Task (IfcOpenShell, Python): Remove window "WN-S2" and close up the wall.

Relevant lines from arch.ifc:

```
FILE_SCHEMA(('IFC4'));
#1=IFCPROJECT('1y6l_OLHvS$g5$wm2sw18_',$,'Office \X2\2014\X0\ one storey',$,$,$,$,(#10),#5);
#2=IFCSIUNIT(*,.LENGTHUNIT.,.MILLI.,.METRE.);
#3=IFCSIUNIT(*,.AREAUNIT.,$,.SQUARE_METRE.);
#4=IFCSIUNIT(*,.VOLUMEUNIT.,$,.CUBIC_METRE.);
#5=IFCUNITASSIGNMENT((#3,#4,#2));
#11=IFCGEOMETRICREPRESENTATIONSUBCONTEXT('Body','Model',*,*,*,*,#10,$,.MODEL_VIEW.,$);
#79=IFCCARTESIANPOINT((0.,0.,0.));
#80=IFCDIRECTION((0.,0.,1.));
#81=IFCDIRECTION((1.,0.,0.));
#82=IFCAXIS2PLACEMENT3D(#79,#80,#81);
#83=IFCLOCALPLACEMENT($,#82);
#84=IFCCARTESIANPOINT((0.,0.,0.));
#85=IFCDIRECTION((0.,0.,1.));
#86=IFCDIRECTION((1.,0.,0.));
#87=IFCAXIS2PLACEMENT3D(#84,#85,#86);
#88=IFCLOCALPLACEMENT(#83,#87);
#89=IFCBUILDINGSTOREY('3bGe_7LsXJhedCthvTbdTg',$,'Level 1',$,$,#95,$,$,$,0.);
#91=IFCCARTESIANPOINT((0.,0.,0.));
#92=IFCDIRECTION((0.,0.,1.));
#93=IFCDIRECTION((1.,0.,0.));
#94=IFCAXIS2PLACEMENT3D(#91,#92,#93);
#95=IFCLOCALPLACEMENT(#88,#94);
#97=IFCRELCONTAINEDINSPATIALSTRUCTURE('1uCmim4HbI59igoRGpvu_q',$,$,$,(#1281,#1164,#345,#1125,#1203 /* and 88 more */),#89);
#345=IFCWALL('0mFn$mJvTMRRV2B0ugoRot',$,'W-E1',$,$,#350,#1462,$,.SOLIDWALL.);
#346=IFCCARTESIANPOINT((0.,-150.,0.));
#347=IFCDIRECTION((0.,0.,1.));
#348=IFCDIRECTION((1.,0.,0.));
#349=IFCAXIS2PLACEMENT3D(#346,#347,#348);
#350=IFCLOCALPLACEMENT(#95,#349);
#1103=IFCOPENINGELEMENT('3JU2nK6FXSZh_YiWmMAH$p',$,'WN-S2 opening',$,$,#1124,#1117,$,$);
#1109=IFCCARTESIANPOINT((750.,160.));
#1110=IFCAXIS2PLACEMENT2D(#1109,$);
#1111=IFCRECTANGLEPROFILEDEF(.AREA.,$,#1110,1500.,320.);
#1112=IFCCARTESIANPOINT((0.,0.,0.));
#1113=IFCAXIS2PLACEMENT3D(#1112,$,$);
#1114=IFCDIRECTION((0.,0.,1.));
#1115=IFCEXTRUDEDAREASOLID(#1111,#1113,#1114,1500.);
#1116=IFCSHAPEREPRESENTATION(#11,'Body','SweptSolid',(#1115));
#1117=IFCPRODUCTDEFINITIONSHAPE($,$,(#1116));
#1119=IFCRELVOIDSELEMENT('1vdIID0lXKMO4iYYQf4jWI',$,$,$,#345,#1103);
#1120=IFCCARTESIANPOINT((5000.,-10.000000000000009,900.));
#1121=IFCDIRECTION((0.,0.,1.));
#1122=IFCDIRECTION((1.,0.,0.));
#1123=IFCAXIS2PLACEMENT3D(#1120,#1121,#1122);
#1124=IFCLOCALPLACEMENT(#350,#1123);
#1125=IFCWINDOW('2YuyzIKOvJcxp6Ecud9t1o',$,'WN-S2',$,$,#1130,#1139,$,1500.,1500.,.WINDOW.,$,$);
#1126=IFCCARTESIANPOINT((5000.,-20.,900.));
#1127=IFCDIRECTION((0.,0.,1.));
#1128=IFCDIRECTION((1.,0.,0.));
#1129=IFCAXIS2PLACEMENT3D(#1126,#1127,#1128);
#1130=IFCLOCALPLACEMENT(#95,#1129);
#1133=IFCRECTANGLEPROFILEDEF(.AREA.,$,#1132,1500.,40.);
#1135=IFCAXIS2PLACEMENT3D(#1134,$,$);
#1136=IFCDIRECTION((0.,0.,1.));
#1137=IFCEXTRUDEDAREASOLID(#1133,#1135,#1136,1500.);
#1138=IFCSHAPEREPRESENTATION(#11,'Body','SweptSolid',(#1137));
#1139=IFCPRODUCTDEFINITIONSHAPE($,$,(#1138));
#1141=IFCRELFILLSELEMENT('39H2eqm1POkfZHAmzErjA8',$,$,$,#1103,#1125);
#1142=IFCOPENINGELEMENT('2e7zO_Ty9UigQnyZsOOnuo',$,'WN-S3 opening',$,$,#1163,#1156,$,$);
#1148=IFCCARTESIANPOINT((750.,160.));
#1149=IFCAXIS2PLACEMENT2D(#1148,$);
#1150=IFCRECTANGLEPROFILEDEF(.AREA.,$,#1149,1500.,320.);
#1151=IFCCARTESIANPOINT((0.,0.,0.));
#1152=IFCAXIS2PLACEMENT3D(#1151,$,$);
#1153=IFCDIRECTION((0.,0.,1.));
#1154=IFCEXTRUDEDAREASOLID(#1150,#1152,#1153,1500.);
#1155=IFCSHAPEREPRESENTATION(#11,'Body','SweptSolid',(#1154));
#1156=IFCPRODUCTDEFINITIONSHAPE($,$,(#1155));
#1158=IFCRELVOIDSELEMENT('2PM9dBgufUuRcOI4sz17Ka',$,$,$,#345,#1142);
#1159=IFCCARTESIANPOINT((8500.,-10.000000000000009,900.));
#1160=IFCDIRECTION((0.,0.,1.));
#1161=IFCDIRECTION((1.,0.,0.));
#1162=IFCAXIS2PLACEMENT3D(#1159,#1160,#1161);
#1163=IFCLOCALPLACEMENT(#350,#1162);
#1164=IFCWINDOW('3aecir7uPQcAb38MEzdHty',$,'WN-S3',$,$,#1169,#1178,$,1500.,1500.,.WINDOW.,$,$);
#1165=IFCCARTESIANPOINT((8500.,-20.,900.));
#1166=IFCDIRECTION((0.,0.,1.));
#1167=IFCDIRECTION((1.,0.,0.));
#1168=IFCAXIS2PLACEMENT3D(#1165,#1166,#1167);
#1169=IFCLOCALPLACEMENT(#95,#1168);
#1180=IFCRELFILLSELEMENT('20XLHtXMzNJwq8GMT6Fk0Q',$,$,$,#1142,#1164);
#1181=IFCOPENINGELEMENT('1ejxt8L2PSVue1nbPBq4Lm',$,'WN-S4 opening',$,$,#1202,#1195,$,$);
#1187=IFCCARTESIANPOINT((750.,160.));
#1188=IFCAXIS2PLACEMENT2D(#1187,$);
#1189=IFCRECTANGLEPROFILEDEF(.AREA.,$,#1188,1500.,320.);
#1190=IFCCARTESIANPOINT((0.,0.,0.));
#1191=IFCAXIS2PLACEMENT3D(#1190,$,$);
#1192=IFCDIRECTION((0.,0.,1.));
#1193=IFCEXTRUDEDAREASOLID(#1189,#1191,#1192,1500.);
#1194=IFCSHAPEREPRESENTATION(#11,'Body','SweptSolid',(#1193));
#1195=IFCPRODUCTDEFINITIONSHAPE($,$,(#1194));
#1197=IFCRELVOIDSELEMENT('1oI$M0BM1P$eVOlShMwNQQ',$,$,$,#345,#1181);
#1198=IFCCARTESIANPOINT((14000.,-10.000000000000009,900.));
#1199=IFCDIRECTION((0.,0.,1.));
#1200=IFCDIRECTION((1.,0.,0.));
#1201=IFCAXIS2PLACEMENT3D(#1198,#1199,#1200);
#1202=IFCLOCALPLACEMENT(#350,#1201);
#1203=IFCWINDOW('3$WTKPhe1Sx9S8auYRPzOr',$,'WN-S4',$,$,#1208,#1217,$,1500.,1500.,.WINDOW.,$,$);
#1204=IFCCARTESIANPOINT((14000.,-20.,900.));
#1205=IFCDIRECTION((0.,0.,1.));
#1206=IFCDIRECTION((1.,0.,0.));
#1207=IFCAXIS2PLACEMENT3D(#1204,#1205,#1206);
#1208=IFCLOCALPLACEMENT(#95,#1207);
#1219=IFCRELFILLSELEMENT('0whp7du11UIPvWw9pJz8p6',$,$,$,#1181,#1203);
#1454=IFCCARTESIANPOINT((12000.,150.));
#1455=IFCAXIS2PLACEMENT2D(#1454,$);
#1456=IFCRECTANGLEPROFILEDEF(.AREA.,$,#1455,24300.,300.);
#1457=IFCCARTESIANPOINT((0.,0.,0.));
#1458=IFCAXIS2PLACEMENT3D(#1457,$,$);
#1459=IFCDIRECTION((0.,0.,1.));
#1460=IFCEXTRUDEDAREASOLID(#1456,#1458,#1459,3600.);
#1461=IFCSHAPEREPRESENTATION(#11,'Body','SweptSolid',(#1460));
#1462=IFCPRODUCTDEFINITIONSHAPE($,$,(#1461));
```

```python
import ifcopenshell
import ifcopenshell.api.feature
import ifcopenshell.api.root
import ifcopenshell.geom
import ifcopenshell.util.shape

model = ifcopenshell.open("arch.ifc")
settings = ifcopenshell.geom.settings()


def volume(element):
    """Net volume in cubic metres, openings subtracted."""
    shape = ifcopenshell.geom.create_shape(settings, element)
    return ifcopenshell.util.shape.get_volume(shape.geometry)


window = model.by_guid("2YuyzIKOvJcxp6Ecud9t1o")
opening = window.FillsVoids[0].RelatingOpeningElement
wall = opening.VoidsElements[0].RelatingBuildingElement
before = volume(wall)

ifcopenshell.api.root.remove_product(model, product=window)
ifcopenshell.api.feature.remove_feature(model, feature=opening)

after = volume(wall)

print(f"wall volume {before:.3f} -> {after:.3f} m3")

model.write("arch_v2.ifc")
```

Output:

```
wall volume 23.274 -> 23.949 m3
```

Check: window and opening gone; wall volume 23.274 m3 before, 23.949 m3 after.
